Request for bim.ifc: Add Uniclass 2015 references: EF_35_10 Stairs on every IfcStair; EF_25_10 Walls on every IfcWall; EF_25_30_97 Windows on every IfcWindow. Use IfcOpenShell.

First a look at what the model holds.

```python
import ifcopenshell

model = ifcopenshell.open("bim.ifc")
print(model.schema)
print("classifications:", [c.Name for c in model.by_type("IfcClassification")])
for ifc_class in ("IfcDoor", "IfcRoof", "IfcStair", "IfcWall", "IfcWindow"):
    print(ifc_class, len(model.by_type(ifc_class)))
```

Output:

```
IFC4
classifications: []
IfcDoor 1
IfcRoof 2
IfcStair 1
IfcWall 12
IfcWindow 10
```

```python
import ifcopenshell
import ifcopenshell.api.classification

model = ifcopenshell.open("bim.ifc")

system = ifcopenshell.api.classification.add_classification(model, classification="Uniclass 2015")

codes = {
    "IfcStair": ("EF_35_10", "Stairs"),
    "IfcWall": ("EF_25_10", "Walls"),
    "IfcWindow": ("EF_25_30_97", "Windows"),
}
for ifc_class, (code, name) in codes.items():
    products = model.by_type(ifc_class)
    ifcopenshell.api.classification.add_reference(
        model, products=products, classification=system, identification=code, name=name
    )
    print(code, len(products))

model.write("bim-out.ifc")
```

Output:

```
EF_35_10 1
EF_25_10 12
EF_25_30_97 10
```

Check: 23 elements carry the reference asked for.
